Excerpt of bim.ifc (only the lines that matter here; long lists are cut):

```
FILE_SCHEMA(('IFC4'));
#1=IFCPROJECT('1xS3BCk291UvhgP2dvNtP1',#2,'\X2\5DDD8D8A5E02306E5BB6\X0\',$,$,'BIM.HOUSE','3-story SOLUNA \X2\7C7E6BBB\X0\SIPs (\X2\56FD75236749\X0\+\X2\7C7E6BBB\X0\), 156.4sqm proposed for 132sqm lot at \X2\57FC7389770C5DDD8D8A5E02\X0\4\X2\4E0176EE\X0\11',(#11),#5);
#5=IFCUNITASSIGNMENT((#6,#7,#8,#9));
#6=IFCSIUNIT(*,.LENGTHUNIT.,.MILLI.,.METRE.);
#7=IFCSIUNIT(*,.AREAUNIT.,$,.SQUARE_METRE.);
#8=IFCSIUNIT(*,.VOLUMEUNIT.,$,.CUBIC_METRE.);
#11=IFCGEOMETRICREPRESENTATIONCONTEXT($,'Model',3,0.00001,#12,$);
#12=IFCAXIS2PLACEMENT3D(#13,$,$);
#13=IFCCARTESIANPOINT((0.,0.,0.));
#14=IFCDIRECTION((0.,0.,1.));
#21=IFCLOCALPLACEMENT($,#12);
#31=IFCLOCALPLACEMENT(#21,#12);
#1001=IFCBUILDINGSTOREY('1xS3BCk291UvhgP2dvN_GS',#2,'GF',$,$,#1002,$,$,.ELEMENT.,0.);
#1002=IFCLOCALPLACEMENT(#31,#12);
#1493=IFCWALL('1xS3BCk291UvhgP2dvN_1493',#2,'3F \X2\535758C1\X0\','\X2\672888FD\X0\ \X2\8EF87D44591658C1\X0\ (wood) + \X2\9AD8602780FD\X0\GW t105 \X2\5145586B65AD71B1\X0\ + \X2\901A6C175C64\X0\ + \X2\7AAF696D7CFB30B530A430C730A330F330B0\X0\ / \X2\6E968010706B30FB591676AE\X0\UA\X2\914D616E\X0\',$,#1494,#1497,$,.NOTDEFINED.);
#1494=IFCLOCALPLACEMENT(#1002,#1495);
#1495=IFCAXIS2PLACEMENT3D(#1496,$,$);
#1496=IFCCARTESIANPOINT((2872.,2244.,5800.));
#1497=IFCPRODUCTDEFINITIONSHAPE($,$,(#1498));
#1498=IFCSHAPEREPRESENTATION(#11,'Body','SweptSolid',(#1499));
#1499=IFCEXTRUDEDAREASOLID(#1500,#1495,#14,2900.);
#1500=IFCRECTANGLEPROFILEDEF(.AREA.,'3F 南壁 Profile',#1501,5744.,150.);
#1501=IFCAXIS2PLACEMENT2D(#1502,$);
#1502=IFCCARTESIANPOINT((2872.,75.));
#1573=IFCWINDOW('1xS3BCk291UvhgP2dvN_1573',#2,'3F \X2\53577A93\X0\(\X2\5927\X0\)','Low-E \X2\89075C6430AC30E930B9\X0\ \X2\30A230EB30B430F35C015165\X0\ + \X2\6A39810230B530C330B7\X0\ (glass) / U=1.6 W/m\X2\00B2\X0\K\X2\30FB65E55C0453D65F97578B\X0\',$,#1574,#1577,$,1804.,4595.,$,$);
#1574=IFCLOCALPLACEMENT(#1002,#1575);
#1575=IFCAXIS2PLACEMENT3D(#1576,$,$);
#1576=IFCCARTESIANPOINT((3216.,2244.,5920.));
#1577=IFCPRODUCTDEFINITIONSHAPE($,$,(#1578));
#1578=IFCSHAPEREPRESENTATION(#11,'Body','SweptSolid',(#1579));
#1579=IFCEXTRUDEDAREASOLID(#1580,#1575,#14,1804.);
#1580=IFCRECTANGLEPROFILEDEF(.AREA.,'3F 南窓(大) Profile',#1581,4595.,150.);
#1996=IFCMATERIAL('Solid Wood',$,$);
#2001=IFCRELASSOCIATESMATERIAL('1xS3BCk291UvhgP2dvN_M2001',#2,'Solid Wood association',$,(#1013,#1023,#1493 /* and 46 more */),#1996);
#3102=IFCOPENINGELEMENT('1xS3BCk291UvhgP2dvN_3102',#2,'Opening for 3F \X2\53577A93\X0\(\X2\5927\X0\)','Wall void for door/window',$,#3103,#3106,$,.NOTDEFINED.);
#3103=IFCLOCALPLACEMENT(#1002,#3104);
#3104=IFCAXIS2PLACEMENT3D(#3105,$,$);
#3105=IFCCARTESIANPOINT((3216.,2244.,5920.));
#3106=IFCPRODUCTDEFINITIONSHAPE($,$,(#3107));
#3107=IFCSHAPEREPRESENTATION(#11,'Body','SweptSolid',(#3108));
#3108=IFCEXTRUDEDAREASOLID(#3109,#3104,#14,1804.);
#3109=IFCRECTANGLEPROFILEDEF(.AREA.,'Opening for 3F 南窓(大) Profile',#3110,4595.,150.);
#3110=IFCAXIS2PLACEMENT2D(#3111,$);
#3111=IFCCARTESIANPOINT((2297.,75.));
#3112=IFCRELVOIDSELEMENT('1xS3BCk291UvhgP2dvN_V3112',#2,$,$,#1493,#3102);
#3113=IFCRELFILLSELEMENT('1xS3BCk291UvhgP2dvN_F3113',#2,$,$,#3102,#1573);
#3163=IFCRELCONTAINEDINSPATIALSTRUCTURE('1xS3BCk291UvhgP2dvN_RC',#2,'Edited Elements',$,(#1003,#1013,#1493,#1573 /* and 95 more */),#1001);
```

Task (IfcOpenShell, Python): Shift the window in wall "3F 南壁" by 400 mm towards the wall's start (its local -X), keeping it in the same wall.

```python
import ifcopenshell
import ifcopenshell.api.geometry
import ifcopenshell.util.placement
import ifcopenshell.util.unit

model = ifcopenshell.open("bim.ifc")
unit_scale = ifcopenshell.util.unit.calculate_unit_scale(model)

window = model.by_id(1573)
opening = window.FillsVoids[0].RelatingOpeningElement
wall = opening.VoidsElements[0].RelatingBuildingElement

wall_matrix = ifcopenshell.util.placement.get_local_placement(wall.ObjectPlacement)
shift = wall_matrix[:3, 0] * -0.4 / unit_scale
before = ifcopenshell.util.placement.get_local_placement(window.ObjectPlacement)[:3, 3].copy()

# The window is not placed relative to its opening, so move both.
for product in (opening, window):
    matrix = ifcopenshell.util.placement.get_local_placement(product.ObjectPlacement)
    matrix[:3, 3] += shift
    ifcopenshell.api.geometry.edit_object_placement(model, product=product, matrix=matrix, is_si=False)

after = ifcopenshell.util.placement.get_local_placement(window.ObjectPlacement)[:3, 3]
print("window moved by", (after - before).round(3) + 0.0)

model.write("bim_updated.ifc")
```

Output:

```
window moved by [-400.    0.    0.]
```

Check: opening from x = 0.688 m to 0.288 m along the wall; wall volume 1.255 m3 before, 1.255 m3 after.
